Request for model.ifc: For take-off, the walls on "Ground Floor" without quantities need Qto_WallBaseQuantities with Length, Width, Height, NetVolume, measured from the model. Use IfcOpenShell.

First a look at what the model holds.

```python
import ifcopenshell
import ifcopenshell.util.element
import ifcopenshell.util.unit

model = ifcopenshell.open("model.ifc")
print(model.schema)
for unit_type in ("LENGTHUNIT", "AREAUNIT", "VOLUMEUNIT"):
    print(unit_type, ifcopenshell.util.unit.calculate_unit_scale(model, unit_type))
storey = next(s for s in model.by_type("IfcBuildingStorey") if s.Name == "Ground Floor")
walls = [e for e in ifcopenshell.util.element.get_decomposition(storey) if e.is_a("IfcWall")]
for e in sorted(walls, key=lambda e: e.id()):
    print(e.id(), e.is_a(), e.Name, list(ifcopenshell.util.element.get_psets(e, qtos_only=True)), sep=" | ")
```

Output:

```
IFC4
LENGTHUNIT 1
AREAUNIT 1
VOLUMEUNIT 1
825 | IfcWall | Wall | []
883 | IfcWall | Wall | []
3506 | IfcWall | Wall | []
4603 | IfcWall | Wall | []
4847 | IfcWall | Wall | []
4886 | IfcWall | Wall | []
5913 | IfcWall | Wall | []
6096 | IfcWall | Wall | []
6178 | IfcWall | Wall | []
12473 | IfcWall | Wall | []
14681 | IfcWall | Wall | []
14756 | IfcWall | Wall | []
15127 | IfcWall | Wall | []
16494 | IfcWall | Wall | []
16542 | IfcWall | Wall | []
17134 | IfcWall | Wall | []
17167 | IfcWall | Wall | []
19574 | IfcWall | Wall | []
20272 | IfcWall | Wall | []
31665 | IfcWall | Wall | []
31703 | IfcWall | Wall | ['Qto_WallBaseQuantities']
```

```python
import ifcopenshell
import ifcopenshell.api.pset
import ifcopenshell.geom
import ifcopenshell.util.element
import ifcopenshell.util.shape
import ifcopenshell.util.unit

model = ifcopenshell.open("model.ifc")
unit_scale = ifcopenshell.util.unit.calculate_unit_scale(model)
volume_scale = ifcopenshell.util.unit.calculate_unit_scale(model, "VOLUMEUNIT")
settings = ifcopenshell.geom.settings()

storey = next(s for s in model.by_type("IfcBuildingStorey") if s.Name == "Ground Floor")
walls = [e for e in ifcopenshell.util.element.get_decomposition(storey) if e.is_a("IfcWall")]

for e in sorted(walls, key=lambda e: e.id()):
    if ifcopenshell.util.element.get_psets(e, qtos_only=True, should_inherit=False):
        continue
    # Geometry comes back in metres, in the element's own axes.
    shape = ifcopenshell.geom.create_shape(settings, e)
    values = {
        "Length": ifcopenshell.util.shape.get_x(shape.geometry) / unit_scale,
        "Width": ifcopenshell.util.shape.get_y(shape.geometry) / unit_scale,
        "Height": ifcopenshell.util.shape.get_z(shape.geometry) / unit_scale,
        "NetVolume": ifcopenshell.util.shape.get_volume(shape.geometry) / volume_scale,
    }
    qto = ifcopenshell.api.pset.add_qto(model, product=e, name="Qto_WallBaseQuantities")
    ifcopenshell.api.pset.edit_qto(model, qto=qto, properties=values)
    print(e.id(), {k: round(v, 3) for k, v in values.items()})

model.write("model-out.ifc")
```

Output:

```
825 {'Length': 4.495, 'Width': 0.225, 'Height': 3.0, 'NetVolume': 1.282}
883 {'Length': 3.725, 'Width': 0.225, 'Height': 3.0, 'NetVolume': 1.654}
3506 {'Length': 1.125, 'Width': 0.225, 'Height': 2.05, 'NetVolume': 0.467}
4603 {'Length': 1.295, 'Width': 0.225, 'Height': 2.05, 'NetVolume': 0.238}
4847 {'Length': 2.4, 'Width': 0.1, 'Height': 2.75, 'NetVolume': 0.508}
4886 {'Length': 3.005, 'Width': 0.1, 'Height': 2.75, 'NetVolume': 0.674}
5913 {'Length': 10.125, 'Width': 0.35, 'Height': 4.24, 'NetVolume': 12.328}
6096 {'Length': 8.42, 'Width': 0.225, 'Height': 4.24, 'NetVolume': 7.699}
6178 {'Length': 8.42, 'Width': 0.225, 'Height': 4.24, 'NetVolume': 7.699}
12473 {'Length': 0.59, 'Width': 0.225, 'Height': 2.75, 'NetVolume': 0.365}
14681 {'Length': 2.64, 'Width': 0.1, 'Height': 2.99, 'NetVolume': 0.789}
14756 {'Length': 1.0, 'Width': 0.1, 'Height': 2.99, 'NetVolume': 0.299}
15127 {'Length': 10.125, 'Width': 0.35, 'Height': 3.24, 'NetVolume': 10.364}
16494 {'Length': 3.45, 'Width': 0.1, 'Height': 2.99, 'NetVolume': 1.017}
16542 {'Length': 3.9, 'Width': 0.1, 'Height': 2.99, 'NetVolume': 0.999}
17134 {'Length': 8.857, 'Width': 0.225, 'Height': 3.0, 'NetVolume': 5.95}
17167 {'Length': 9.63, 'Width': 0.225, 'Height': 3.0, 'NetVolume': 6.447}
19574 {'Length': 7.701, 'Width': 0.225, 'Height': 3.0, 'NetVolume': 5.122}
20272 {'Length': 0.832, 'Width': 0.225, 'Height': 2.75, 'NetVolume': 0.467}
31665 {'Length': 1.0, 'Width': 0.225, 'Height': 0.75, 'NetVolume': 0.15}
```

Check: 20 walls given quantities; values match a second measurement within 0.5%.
